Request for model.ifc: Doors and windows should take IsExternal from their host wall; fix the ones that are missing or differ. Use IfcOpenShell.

First a look at what the model holds.

```python
import ifcopenshell
import ifcopenshell.util.element

model = ifcopenshell.open("model.ifc")
print(model.schema)
seen = {}
for e in model.by_type("IfcDoor") + model.by_type("IfcWindow"):
    if not e.FillsVoids:
        continue
    host = e.FillsVoids[0].RelatingOpeningElement.VoidsElements[0].RelatingBuildingElement
    own = ifcopenshell.util.element.get_pset(e, f"Pset_{e.is_a()[3:].removesuffix('StandardCase')}Common", "IsExternal")
    wall = ifcopenshell.util.element.get_pset(host, "Pset_WallCommon", "IsExternal")
    seen[e.is_a(), own, wall] = seen.get((e.is_a(), own, wall), 0) + 1
for (cls, own, wall), count in sorted(seen.items(), key=str):
    print(count, cls, "IsExternal:", own, "| host wall:", wall)
```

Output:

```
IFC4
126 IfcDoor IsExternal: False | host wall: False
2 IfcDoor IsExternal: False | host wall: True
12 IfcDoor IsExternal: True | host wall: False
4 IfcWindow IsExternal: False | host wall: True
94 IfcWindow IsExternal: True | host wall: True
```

```python
import ifcopenshell
import ifcopenshell.api.pset
import ifcopenshell.util.element

model = ifcopenshell.open("model.ifc")

count = 0
for ifc_class, pset_name in (("IfcDoor", "Pset_DoorCommon"), ("IfcWindow", "Pset_WindowCommon")):
    for e in model.by_type(ifc_class):
        if not e.FillsVoids:
            continue
        host = e.FillsVoids[0].RelatingOpeningElement.VoidsElements[0].RelatingBuildingElement
        external = ifcopenshell.util.element.get_pset(host, "Pset_WallCommon", "IsExternal")
        if external is None or ifcopenshell.util.element.get_pset(e, pset_name, "IsExternal") == external:
            continue
        pset = ifcopenshell.api.pset.add_pset(model, product=e, name=pset_name)
        ifcopenshell.api.pset.edit_pset(model, pset=pset, properties={"IsExternal": external})
        count += 1

print(count, "updated")

model.write("model_edited.ifc")
```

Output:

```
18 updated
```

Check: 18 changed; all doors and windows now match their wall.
